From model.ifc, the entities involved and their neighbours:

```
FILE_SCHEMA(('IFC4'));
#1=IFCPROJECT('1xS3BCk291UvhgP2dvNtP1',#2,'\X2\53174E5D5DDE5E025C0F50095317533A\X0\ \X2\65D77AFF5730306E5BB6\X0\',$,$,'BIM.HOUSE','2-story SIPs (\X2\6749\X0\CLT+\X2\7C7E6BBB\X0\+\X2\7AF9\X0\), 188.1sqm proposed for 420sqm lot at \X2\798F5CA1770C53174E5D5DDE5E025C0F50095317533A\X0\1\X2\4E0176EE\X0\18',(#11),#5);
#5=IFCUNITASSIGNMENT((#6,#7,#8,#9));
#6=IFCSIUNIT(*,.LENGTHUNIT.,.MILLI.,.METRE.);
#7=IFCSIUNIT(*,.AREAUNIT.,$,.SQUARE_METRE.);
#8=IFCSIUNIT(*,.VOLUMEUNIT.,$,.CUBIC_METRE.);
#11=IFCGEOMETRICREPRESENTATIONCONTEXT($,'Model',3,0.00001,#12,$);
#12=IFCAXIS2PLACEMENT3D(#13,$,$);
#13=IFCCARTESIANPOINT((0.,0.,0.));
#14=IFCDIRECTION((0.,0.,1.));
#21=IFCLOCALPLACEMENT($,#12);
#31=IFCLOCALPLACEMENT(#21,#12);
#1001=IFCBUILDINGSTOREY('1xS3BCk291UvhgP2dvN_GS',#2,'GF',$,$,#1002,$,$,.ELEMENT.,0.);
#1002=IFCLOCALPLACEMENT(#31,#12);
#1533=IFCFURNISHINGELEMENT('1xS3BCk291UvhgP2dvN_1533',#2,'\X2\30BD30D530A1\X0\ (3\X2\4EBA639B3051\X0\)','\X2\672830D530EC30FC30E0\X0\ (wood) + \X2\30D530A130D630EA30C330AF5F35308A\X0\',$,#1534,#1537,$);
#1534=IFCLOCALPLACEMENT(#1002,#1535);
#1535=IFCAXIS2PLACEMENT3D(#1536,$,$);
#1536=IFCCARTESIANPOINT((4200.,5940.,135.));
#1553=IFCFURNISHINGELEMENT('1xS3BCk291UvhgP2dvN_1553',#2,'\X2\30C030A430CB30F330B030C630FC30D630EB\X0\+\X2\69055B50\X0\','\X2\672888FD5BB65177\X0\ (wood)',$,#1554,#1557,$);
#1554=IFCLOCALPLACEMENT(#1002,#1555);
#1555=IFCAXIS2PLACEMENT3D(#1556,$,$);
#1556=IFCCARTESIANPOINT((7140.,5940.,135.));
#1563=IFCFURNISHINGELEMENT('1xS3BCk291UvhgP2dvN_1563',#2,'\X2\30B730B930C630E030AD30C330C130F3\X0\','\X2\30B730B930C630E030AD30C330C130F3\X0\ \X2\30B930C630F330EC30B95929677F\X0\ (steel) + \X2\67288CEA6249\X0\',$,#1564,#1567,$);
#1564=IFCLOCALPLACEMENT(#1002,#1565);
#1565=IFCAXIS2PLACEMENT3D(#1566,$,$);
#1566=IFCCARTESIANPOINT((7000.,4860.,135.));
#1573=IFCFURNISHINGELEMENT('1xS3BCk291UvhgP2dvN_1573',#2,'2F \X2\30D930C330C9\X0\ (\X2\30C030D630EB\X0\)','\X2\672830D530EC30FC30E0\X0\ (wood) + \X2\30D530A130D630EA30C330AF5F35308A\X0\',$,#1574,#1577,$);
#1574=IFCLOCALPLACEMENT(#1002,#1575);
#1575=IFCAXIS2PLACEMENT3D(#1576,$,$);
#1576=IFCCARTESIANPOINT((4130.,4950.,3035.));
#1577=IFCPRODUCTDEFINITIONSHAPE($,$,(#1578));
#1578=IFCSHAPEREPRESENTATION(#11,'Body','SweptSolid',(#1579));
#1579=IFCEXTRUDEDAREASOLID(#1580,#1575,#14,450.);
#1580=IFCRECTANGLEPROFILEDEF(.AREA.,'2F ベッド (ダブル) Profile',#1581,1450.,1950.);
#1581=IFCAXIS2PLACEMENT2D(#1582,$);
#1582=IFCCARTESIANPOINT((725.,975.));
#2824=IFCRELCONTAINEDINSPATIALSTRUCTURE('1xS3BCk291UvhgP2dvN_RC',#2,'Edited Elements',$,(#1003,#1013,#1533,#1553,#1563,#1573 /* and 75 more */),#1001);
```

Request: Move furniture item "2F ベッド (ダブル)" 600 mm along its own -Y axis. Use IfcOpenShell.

```python
import ifcopenshell
import ifcopenshell.api.geometry
import ifcopenshell.util.placement

model = ifcopenshell.open("model.ifc")

item = model.by_guid("1xS3BCk291UvhgP2dvN_1573")
matrix = ifcopenshell.util.placement.get_local_placement(item.ObjectPlacement)
matrix[:3, 3] -= matrix[:3, 1] * 600.0
ifcopenshell.api.geometry.edit_object_placement(model, product=item, matrix=matrix, is_si=False)

print(ifcopenshell.util.placement.get_local_placement(item.ObjectPlacement).round(3) + 0.0)

model.write("model_v2.ifc")
```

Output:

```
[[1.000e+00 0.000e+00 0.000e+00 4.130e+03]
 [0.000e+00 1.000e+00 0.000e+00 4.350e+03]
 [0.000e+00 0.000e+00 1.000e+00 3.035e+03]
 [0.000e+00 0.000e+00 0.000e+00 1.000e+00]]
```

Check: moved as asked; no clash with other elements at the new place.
